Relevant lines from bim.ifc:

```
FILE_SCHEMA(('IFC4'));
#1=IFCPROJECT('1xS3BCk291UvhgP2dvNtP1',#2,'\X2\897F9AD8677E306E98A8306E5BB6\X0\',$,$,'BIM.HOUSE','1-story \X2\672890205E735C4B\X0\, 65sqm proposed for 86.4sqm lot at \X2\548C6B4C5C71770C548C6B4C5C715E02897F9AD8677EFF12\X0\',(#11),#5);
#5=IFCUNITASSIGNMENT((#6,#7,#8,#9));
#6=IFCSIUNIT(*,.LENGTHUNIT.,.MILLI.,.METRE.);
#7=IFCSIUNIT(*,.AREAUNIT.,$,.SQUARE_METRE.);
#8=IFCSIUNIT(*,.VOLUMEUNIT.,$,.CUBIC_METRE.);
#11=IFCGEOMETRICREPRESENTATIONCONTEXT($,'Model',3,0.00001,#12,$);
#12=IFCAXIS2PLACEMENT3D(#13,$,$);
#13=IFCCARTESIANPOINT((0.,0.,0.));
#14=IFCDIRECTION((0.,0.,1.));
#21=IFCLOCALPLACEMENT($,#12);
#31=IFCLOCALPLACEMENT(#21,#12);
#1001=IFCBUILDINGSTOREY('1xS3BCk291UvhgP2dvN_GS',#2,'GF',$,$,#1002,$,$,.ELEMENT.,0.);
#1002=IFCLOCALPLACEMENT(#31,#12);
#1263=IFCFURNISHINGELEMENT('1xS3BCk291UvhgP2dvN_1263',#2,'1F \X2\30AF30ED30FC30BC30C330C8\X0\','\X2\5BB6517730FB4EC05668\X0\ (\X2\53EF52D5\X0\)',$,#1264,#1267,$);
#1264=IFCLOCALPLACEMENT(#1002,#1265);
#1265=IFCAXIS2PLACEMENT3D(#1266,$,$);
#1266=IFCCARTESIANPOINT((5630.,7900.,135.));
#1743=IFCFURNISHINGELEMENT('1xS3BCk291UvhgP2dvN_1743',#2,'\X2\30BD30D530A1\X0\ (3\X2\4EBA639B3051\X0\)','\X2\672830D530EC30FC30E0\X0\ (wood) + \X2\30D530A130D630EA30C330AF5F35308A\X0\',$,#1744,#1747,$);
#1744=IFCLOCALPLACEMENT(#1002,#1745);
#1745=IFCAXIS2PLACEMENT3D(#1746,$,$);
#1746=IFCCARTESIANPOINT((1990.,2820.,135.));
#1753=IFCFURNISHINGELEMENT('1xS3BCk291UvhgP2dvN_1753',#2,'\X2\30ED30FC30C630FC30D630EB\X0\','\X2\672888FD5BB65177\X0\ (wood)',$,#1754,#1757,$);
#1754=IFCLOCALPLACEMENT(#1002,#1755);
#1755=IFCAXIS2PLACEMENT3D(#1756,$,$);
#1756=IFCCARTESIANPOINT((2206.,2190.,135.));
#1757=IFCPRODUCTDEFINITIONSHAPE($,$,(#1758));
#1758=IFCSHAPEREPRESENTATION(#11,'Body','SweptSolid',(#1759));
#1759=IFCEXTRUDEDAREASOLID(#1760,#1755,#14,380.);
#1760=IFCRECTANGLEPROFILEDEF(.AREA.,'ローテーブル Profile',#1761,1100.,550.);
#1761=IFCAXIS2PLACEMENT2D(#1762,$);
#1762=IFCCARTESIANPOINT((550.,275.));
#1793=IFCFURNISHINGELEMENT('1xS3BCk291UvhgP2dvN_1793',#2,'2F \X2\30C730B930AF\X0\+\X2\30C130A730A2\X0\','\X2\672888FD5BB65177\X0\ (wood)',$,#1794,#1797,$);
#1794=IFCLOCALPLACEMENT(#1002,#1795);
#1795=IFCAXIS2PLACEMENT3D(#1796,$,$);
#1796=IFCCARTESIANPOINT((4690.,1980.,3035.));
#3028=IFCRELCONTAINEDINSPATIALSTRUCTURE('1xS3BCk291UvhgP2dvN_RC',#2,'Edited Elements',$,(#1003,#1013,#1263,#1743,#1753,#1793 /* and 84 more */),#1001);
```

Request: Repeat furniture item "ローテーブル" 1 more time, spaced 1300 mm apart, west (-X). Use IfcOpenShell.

```python
import numpy as np
import ifcopenshell
import ifcopenshell.api.geometry
import ifcopenshell.api.root
import ifcopenshell.util.element
import ifcopenshell.util.placement

model = ifcopenshell.open("bim.ifc")


def reuse_history(source, copy):
    """copy_class also copies each property set's owner history, people and application; keep the originals."""
    for rel in copy.IsDefinedBy:
        if rel.is_a("IfcRelDefinesByProperties") and (history := rel.RelatingPropertyDefinition.OwnerHistory):
            rel.RelatingPropertyDefinition.OwnerHistory = source.OwnerHistory
            ifcopenshell.util.element.remove_deep2(model, history)


source = model.by_guid("1xS3BCk291UvhgP2dvN_1753")
base = ifcopenshell.util.placement.get_local_placement(source.ObjectPlacement)
step = np.array([-1.0, 0.0, 0.0]) * 1300.0

for i in range(1, 2):
    copy = ifcopenshell.api.root.copy_class(model, product=source)
    copy.Representation = ifcopenshell.util.element.copy_deep(
        model, source.Representation, exclude=["IfcGeometricRepresentationContext", "IfcRepresentationMap"]
    )
    reuse_history(source, copy)
    matrix = base.copy()
    matrix[:3, 3] += i * step
    print("added at", matrix[:3, 3].round(3) + 0.0)
    ifcopenshell.api.geometry.edit_object_placement(model, product=copy, matrix=matrix, is_si=False)

model.write("bim_rev.ifc")
```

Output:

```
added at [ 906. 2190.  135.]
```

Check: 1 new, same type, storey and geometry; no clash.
